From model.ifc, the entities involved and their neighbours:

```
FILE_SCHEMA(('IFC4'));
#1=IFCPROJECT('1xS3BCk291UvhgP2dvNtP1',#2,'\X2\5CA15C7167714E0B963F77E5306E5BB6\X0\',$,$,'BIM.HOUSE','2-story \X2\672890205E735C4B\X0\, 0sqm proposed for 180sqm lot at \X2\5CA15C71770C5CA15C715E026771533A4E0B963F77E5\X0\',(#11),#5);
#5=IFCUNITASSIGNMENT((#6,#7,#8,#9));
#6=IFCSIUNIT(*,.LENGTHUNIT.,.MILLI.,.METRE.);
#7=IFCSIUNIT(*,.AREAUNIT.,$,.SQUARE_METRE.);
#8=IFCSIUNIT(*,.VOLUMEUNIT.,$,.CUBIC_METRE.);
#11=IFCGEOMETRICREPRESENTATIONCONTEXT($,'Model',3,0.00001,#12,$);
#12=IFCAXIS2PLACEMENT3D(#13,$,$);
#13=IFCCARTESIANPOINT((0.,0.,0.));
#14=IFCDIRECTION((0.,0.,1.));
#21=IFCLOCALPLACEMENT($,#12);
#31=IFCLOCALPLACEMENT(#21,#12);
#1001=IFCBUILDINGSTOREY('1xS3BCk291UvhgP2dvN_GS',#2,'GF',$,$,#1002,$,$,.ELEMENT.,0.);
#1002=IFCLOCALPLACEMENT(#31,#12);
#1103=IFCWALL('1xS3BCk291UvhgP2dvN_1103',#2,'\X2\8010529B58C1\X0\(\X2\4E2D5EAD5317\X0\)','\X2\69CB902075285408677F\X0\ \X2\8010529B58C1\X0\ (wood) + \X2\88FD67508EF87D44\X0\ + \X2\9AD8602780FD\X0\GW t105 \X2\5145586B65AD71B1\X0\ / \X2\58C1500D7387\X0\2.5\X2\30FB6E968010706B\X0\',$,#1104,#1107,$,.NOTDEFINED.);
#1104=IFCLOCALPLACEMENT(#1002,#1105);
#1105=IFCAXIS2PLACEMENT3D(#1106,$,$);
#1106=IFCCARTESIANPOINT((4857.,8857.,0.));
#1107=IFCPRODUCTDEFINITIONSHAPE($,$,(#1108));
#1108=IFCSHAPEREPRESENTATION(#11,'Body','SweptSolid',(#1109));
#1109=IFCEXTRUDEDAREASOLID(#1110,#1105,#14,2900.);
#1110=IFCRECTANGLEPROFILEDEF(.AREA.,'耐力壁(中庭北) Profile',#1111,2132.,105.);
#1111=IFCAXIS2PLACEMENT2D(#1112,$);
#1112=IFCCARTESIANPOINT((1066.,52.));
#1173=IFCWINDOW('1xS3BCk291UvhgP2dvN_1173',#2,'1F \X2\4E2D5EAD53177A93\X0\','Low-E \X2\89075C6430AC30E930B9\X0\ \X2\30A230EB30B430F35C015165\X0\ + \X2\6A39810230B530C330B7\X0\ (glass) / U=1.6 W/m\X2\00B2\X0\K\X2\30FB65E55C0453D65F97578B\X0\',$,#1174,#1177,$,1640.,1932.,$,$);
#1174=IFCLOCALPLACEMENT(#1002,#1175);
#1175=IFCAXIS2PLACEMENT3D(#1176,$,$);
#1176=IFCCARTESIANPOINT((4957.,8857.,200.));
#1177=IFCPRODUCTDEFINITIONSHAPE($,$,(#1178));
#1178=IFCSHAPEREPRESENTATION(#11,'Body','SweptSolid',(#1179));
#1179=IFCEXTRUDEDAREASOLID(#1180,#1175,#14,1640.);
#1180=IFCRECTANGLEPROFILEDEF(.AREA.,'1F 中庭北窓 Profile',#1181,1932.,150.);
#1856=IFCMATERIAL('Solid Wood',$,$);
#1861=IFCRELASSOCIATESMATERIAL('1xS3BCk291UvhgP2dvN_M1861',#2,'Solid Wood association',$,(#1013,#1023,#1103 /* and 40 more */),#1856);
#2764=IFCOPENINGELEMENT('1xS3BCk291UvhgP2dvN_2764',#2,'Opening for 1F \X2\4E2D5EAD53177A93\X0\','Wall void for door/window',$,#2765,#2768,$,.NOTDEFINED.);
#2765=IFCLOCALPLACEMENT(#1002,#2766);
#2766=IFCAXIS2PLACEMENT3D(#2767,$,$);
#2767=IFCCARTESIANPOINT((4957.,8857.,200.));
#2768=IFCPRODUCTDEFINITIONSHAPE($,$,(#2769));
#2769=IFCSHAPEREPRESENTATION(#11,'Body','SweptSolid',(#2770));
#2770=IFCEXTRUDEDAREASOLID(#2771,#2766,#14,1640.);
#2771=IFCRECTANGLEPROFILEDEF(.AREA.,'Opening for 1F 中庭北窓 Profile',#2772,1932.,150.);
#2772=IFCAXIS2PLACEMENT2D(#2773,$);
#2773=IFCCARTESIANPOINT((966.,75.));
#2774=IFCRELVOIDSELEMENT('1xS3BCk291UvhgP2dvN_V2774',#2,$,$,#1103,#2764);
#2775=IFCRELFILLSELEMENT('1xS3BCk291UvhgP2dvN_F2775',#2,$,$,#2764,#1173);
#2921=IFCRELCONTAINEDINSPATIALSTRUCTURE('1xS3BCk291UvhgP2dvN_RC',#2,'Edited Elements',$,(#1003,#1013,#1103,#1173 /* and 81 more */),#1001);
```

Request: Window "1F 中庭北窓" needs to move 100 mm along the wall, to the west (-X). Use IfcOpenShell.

```python
import ifcopenshell
import ifcopenshell.api.geometry
import ifcopenshell.util.placement

model = ifcopenshell.open("model.ifc")

window = model.by_guid("1xS3BCk291UvhgP2dvN_1173")
opening = window.FillsVoids[0].RelatingOpeningElement
wall = opening.VoidsElements[0].RelatingBuildingElement

wall_matrix = ifcopenshell.util.placement.get_local_placement(wall.ObjectPlacement)
shift = wall_matrix[:3, 0] * -100.0
before = ifcopenshell.util.placement.get_local_placement(window.ObjectPlacement)[:3, 3].copy()

# The window is not placed relative to its opening, so move both.
for product in (opening, window):
    matrix = ifcopenshell.util.placement.get_local_placement(product.ObjectPlacement)
    matrix[:3, 3] += shift
    ifcopenshell.api.geometry.edit_object_placement(model, product=product, matrix=matrix, is_si=False)

after = ifcopenshell.util.placement.get_local_placement(window.ObjectPlacement)[:3, 3]
print("window moved by", (after - before).round(3) + 0.0)

model.write("model_edited.ifc")
```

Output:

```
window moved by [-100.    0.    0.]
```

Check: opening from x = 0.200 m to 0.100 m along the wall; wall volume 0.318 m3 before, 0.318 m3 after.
